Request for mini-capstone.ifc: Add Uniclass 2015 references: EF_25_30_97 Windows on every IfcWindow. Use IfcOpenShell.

First a look at what the model holds.

```python
import ifcopenshell

model = ifcopenshell.open("mini-capstone.ifc")
print(model.schema)
print("classifications:", [c.Name for c in model.by_type("IfcClassification")])
for ifc_class in ("IfcDoor", "IfcRoof", "IfcStair", "IfcWall", "IfcWindow"):
    print(ifc_class, len(model.by_type(ifc_class)))
```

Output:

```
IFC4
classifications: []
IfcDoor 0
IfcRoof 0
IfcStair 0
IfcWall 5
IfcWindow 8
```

```python
import ifcopenshell
import ifcopenshell.api.classification

model = ifcopenshell.open("mini-capstone.ifc")

system = ifcopenshell.api.classification.add_classification(model, classification="Uniclass 2015")

codes = {
    "IfcWindow": ("EF_25_30_97", "Windows"),
}
for ifc_class, (code, name) in codes.items():
    products = model.by_type(ifc_class)
    ifcopenshell.api.classification.add_reference(
        model, products=products, classification=system, identification=code, name=name
    )
    print(code, len(products))

model.write("mini-capstone_updated.ifc")
```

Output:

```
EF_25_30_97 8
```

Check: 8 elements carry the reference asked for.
